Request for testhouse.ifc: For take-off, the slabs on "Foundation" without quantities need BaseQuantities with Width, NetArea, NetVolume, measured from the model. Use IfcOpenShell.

First a look at what the model holds.

```python
import ifcopenshell
import ifcopenshell.util.element
import ifcopenshell.util.unit

model = ifcopenshell.open("testhouse.ifc")
print(model.schema)
for unit_type in ("LENGTHUNIT", "AREAUNIT", "VOLUMEUNIT"):
    print(unit_type, ifcopenshell.util.unit.calculate_unit_scale(model, unit_type))
storey = next(s for s in model.by_type("IfcBuildingStorey") if s.Name == "Foundation")
slabs = [e for e in ifcopenshell.util.element.get_decomposition(storey) if e.is_a("IfcSlab")]
for e in sorted(slabs, key=lambda e: e.id()):
    print(e.id(), e.is_a(), e.Name, list(ifcopenshell.util.element.get_psets(e, qtos_only=True)), sep=" | ")
```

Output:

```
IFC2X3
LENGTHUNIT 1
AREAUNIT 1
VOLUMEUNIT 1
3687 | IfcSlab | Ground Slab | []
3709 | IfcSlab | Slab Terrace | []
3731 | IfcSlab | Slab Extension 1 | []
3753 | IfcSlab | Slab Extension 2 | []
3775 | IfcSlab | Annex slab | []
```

```python
import ifcopenshell
import ifcopenshell.api.pset
import ifcopenshell.geom
import ifcopenshell.util.element
import ifcopenshell.util.shape
import ifcopenshell.util.unit

model = ifcopenshell.open("testhouse.ifc")
unit_scale = ifcopenshell.util.unit.calculate_unit_scale(model)
area_scale = ifcopenshell.util.unit.calculate_unit_scale(model, "AREAUNIT")
volume_scale = ifcopenshell.util.unit.calculate_unit_scale(model, "VOLUMEUNIT")
settings = ifcopenshell.geom.settings()

storey = next(s for s in model.by_type("IfcBuildingStorey") if s.Name == "Foundation")
slabs = [e for e in ifcopenshell.util.element.get_decomposition(storey) if e.is_a("IfcSlab")]

for e in sorted(slabs, key=lambda e: e.id()):
    if ifcopenshell.util.element.get_psets(e, qtos_only=True, should_inherit=False):
        continue
    # Geometry comes back in metres, in the element's own axes.
    shape = ifcopenshell.geom.create_shape(settings, e)
    values = {
        "Width": ifcopenshell.util.shape.get_z(shape.geometry) / unit_scale,
        "NetArea": ifcopenshell.util.shape.get_footprint_area(shape.geometry) / area_scale,
        "NetVolume": ifcopenshell.util.shape.get_volume(shape.geometry) / volume_scale,
    }
    qto = ifcopenshell.api.pset.add_qto(model, product=e, name="BaseQuantities")
    ifcopenshell.api.pset.edit_qto(model, qto=qto, properties=values)
    print(e.id(), {k: round(v, 3) for k, v in values.items()})

model.write("testhouse_rev.ifc")
```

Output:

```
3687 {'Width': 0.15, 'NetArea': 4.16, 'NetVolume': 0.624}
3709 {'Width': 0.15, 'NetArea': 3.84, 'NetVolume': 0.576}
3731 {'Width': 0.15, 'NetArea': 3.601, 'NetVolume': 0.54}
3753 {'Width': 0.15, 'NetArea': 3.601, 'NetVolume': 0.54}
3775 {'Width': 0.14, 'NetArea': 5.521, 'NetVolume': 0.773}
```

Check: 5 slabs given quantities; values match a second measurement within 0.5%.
